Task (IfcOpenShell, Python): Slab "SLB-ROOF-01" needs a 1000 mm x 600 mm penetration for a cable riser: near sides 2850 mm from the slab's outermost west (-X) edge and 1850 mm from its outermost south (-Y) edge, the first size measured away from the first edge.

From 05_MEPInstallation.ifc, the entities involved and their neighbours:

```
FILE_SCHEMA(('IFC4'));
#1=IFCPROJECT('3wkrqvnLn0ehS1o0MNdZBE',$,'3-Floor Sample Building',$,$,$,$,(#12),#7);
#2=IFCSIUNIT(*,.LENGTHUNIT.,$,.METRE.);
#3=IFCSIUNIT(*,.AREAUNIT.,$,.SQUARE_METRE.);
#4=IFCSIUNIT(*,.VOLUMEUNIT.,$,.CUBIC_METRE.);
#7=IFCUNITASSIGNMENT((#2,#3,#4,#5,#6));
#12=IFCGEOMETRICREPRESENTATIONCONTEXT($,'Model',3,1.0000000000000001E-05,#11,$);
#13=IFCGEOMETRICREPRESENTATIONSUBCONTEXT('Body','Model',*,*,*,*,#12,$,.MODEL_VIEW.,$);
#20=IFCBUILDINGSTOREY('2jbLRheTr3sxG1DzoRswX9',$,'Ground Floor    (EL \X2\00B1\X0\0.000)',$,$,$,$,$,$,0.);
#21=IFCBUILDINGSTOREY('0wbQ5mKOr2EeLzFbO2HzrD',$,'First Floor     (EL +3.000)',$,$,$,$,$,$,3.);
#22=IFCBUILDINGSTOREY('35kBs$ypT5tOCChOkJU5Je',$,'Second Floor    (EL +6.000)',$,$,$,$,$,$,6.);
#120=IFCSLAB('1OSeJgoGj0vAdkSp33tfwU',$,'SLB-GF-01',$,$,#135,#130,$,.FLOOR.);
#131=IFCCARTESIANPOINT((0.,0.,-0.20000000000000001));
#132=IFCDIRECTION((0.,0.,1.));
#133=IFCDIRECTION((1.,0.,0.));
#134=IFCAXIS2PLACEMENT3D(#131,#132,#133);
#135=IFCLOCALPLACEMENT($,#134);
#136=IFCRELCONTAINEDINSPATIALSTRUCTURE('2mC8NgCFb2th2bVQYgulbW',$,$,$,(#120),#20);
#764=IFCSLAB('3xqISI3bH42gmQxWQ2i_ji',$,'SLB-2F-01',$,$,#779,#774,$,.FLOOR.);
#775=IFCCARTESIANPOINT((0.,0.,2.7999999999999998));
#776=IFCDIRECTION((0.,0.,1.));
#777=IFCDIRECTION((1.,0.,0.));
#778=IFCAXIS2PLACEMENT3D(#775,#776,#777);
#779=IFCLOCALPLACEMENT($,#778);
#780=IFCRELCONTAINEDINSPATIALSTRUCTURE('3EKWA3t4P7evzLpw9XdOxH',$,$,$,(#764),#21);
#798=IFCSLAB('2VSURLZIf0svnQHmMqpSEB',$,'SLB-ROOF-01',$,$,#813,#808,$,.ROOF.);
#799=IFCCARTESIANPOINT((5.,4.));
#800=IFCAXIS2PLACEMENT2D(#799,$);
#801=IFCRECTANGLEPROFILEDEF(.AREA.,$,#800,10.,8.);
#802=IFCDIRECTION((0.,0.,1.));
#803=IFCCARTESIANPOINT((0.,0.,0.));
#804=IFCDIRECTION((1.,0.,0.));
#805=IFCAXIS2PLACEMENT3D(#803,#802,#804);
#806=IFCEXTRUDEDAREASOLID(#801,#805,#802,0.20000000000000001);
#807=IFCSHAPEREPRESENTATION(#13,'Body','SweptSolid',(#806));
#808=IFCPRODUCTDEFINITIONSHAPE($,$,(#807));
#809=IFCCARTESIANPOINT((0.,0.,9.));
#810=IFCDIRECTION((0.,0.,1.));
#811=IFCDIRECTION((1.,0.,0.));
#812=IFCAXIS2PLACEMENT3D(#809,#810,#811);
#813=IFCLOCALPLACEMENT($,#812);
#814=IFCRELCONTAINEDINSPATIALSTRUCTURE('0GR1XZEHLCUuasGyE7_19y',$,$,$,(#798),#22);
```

```python
import numpy as np
import ifcopenshell
import ifcopenshell.api.feature
import ifcopenshell.api.geometry
import ifcopenshell.api.root
import ifcopenshell.geom
import ifcopenshell.util.placement
import ifcopenshell.util.representation
import ifcopenshell.util.shape
import ifcopenshell.util.unit

model = ifcopenshell.open("05_MEPInstallation.ifc")
unit_scale = ifcopenshell.util.unit.calculate_unit_scale(model)
settings = ifcopenshell.geom.settings()


def volume(element):
    """Net volume in cubic metres, openings subtracted."""
    shape = ifcopenshell.geom.create_shape(settings, element)
    return ifcopenshell.util.shape.get_volume(shape.geometry)


slab = model.by_guid("2VSURLZIf0svnQHmMqpSEB")
before = volume(slab)

# Extent in the slab's own axes, in metres. The edges named are its -X and -Y sides.
slab_shape = ifcopenshell.geom.create_shape(settings, slab)
vertices = ifcopenshell.util.shape.get_vertices(slab_shape.geometry)
x_min, y_min, bottom = vertices.min(axis=0)
top = vertices[:, 2].max()

opening = ifcopenshell.api.root.create_entity(model, ifc_class="IfcOpeningElement", name="Cable riser opening", predefined_type="OPENING")
context = ifcopenshell.util.representation.get_context(model, "Model", "Body", "MODEL_VIEW")
width, depth = 1, 0.6
outline = [(0.0, 0.0), (width, 0.0), (width, depth), (0.0, depth), (0.0, 0.0)]
# Overshoot both faces by 50 mm so the cut is clean.
shape = ifcopenshell.api.geometry.add_slab_representation(
    model, context=context, depth=top - bottom + 0.1, polyline=outline
)
ifcopenshell.api.geometry.assign_representation(model, product=opening, representation=shape)

matrix = ifcopenshell.util.placement.get_local_placement(slab.ObjectPlacement)
matrix[:, 3] = matrix @ np.append(np.array([x_min + 2.85, y_min + 1.85, bottom - 0.05]) / unit_scale, 1.0)
ifcopenshell.api.geometry.edit_object_placement(model, product=opening, matrix=matrix, is_si=False)
ifcopenshell.api.feature.add_feature(model, feature=opening, element=slab)

after = volume(slab)

print(f"slab volume {before:.3f} -> {after:.3f} m3")

model.write("05_MEPInstallation_edited.ifc")
```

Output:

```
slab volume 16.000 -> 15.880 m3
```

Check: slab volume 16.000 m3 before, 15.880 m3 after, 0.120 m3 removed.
